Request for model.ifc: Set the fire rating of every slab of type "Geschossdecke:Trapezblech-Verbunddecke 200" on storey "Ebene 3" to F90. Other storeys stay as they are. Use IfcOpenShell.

First a look at what the model holds.

```python
import ifcopenshell
import ifcopenshell.util.element

model = ifcopenshell.open("model.ifc")
print(model.schema)
storey = next(s for s in model.by_type("IfcBuildingStorey") if s.Name == "Ebene 3")
slabs = [e for e in ifcopenshell.util.element.get_decomposition(storey) if e.is_a("IfcSlab")]
seen = {}
for e in slabs:
    element_type = ifcopenshell.util.element.get_type(e)
    key = (element_type.Name if element_type != e and element_type else None, ifcopenshell.util.element.get_pset(e, "Pset_SlabCommon", "FireRating"))
    seen[key] = seen.get(key, 0) + 1
for (name, value), count in sorted(seen.items(), key=str):
    print(count, "x", name, "|", value)
```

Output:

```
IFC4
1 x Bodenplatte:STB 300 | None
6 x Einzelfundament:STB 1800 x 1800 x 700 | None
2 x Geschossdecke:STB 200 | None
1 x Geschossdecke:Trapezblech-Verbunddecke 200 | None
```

```python
import ifcopenshell
import ifcopenshell.api.pset
import ifcopenshell.util.element

model = ifcopenshell.open("model.ifc")

storey = next(s for s in model.by_type("IfcBuildingStorey") if s.Name == "Ebene 3")
slabs = [e for e in ifcopenshell.util.element.get_decomposition(storey) if e.is_a("IfcSlab")]

count = 0
for e in slabs:
    element_type = ifcopenshell.util.element.get_type(e)
    if element_type in (None, e) or element_type.Name != "Geschossdecke:Trapezblech-Verbunddecke 200":
        continue
    # add_pset returns the element's existing set when there is one.
    pset = ifcopenshell.api.pset.add_pset(model, product=e, name="Pset_SlabCommon")
    ifcopenshell.api.pset.edit_pset(model, pset=pset, properties={"FireRating": "F90"})
    count += 1

print(count, "slabs updated")

model.write("model_rev.ifc")
```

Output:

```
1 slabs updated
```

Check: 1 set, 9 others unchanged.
